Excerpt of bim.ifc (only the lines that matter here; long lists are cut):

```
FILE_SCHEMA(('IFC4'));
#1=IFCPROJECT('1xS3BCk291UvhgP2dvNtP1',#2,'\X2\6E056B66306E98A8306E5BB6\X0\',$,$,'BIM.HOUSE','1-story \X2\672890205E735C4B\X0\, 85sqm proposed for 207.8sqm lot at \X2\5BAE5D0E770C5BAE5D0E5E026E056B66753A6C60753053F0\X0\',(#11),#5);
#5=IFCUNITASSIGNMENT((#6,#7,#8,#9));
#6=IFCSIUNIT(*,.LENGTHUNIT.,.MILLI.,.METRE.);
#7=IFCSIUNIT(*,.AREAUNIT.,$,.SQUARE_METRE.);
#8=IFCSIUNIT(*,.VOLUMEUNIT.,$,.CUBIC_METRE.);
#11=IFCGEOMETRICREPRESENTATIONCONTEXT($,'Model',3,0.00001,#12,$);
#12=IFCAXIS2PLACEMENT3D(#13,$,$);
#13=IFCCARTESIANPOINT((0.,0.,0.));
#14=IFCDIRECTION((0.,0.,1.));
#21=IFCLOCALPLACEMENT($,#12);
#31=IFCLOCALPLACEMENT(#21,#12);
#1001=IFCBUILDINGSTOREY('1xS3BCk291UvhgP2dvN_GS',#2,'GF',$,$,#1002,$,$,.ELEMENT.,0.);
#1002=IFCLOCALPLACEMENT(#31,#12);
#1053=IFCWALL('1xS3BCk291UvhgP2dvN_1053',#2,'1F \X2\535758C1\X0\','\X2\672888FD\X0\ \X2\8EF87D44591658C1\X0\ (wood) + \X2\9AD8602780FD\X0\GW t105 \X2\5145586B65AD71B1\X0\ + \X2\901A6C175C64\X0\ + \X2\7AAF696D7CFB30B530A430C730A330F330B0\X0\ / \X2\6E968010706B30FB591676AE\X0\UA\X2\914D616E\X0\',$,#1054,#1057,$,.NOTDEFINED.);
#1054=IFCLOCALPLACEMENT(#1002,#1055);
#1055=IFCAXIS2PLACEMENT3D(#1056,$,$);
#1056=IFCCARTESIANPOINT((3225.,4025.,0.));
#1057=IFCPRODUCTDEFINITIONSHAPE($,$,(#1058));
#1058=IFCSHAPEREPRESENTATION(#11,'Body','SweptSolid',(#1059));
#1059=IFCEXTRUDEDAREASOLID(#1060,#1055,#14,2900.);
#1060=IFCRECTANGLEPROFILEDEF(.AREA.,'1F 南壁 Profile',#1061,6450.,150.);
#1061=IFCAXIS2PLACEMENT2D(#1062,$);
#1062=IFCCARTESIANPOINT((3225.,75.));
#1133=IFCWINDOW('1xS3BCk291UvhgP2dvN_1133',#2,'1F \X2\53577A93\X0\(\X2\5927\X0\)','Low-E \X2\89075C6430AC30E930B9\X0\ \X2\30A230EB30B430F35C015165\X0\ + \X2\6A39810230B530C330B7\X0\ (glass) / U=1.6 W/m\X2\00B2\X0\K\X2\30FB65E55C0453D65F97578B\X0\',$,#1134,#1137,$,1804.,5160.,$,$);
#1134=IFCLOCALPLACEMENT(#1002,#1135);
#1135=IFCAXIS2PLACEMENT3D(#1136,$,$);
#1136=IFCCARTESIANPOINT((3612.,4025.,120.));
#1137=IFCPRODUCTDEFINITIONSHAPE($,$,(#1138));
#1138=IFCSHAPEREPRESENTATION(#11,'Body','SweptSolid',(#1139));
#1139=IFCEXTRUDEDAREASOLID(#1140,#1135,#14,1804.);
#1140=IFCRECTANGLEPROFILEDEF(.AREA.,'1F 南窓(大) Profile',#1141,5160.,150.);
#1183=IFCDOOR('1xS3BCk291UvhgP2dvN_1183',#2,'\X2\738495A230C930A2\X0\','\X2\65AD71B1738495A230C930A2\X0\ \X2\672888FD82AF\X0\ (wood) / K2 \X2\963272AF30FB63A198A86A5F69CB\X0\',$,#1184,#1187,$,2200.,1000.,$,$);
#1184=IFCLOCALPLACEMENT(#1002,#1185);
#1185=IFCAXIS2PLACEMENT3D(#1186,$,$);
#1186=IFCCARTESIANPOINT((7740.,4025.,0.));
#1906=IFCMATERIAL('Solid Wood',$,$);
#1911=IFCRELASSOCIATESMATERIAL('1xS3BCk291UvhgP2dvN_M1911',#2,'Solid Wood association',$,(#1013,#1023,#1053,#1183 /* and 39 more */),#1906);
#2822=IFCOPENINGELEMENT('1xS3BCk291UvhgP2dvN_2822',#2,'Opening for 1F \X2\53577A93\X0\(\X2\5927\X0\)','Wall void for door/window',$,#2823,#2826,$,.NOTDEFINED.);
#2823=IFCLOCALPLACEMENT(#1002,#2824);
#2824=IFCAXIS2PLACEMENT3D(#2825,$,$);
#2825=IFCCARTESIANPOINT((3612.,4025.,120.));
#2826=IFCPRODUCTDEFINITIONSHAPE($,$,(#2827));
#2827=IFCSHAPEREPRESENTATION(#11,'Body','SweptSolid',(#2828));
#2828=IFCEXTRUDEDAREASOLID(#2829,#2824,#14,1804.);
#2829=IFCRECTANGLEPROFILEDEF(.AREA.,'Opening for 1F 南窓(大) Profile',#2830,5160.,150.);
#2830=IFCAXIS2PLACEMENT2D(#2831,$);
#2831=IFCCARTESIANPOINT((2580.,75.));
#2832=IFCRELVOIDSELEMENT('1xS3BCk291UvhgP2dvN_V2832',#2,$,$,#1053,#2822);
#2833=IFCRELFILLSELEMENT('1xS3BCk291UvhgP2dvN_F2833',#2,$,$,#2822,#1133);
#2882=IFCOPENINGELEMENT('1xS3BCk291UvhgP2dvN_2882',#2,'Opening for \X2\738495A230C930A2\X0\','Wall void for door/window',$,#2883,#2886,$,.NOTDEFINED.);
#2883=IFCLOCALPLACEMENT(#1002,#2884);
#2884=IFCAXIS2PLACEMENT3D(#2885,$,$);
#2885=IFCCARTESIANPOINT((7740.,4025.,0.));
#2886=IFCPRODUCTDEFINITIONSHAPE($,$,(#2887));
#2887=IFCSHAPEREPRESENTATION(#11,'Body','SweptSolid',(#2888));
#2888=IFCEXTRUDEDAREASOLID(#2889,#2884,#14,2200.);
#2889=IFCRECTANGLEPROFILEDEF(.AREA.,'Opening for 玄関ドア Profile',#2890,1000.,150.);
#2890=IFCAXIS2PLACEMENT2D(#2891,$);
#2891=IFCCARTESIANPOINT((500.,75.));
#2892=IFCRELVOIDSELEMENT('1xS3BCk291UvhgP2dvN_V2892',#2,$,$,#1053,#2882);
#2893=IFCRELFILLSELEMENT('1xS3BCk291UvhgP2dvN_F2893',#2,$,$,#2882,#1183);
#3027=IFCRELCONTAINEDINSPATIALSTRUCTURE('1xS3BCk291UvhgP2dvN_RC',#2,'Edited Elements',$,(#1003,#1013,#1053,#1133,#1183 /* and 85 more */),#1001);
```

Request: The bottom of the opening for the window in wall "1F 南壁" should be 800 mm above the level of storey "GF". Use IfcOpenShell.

```python
import numpy as np
import ifcopenshell
import ifcopenshell.api.geometry
import ifcopenshell.geom
import ifcopenshell.util.element
import ifcopenshell.util.placement
import ifcopenshell.util.shape
import ifcopenshell.util.unit

model = ifcopenshell.open("bim.ifc")
unit_scale = ifcopenshell.util.unit.calculate_unit_scale(model)

window = model.by_guid("1xS3BCk291UvhgP2dvN_1133")
opening = window.FillsVoids[0].RelatingOpeningElement
storey = ifcopenshell.util.element.get_container(window, ifc_class="IfcBuildingStorey")
level = ifcopenshell.util.placement.get_local_placement(storey.ObjectPlacement)[2, 3]

# The opening's origin need not be at the sill, so measure its lowest point.
shape = ifcopenshell.geom.create_shape(ifcopenshell.geom.settings(), opening)
bottom = ifcopenshell.util.shape.get_shape_bottom_elevation(shape, shape.geometry) / unit_scale
dz = level + 800.0 - bottom

shift = np.array([0.0, 0.0, dz])
# The window is not placed relative to its opening, so move both.
for product in (opening, window):
    matrix = ifcopenshell.util.placement.get_local_placement(product.ObjectPlacement)
    matrix[:3, 3] += shift
    ifcopenshell.api.geometry.edit_object_placement(model, product=product, matrix=matrix, is_si=False)

print(f"moved by {dz * unit_scale:+.3f} m")

model.write("bim_edited.ifc")
```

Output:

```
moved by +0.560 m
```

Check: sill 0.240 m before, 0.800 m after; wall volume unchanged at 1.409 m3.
